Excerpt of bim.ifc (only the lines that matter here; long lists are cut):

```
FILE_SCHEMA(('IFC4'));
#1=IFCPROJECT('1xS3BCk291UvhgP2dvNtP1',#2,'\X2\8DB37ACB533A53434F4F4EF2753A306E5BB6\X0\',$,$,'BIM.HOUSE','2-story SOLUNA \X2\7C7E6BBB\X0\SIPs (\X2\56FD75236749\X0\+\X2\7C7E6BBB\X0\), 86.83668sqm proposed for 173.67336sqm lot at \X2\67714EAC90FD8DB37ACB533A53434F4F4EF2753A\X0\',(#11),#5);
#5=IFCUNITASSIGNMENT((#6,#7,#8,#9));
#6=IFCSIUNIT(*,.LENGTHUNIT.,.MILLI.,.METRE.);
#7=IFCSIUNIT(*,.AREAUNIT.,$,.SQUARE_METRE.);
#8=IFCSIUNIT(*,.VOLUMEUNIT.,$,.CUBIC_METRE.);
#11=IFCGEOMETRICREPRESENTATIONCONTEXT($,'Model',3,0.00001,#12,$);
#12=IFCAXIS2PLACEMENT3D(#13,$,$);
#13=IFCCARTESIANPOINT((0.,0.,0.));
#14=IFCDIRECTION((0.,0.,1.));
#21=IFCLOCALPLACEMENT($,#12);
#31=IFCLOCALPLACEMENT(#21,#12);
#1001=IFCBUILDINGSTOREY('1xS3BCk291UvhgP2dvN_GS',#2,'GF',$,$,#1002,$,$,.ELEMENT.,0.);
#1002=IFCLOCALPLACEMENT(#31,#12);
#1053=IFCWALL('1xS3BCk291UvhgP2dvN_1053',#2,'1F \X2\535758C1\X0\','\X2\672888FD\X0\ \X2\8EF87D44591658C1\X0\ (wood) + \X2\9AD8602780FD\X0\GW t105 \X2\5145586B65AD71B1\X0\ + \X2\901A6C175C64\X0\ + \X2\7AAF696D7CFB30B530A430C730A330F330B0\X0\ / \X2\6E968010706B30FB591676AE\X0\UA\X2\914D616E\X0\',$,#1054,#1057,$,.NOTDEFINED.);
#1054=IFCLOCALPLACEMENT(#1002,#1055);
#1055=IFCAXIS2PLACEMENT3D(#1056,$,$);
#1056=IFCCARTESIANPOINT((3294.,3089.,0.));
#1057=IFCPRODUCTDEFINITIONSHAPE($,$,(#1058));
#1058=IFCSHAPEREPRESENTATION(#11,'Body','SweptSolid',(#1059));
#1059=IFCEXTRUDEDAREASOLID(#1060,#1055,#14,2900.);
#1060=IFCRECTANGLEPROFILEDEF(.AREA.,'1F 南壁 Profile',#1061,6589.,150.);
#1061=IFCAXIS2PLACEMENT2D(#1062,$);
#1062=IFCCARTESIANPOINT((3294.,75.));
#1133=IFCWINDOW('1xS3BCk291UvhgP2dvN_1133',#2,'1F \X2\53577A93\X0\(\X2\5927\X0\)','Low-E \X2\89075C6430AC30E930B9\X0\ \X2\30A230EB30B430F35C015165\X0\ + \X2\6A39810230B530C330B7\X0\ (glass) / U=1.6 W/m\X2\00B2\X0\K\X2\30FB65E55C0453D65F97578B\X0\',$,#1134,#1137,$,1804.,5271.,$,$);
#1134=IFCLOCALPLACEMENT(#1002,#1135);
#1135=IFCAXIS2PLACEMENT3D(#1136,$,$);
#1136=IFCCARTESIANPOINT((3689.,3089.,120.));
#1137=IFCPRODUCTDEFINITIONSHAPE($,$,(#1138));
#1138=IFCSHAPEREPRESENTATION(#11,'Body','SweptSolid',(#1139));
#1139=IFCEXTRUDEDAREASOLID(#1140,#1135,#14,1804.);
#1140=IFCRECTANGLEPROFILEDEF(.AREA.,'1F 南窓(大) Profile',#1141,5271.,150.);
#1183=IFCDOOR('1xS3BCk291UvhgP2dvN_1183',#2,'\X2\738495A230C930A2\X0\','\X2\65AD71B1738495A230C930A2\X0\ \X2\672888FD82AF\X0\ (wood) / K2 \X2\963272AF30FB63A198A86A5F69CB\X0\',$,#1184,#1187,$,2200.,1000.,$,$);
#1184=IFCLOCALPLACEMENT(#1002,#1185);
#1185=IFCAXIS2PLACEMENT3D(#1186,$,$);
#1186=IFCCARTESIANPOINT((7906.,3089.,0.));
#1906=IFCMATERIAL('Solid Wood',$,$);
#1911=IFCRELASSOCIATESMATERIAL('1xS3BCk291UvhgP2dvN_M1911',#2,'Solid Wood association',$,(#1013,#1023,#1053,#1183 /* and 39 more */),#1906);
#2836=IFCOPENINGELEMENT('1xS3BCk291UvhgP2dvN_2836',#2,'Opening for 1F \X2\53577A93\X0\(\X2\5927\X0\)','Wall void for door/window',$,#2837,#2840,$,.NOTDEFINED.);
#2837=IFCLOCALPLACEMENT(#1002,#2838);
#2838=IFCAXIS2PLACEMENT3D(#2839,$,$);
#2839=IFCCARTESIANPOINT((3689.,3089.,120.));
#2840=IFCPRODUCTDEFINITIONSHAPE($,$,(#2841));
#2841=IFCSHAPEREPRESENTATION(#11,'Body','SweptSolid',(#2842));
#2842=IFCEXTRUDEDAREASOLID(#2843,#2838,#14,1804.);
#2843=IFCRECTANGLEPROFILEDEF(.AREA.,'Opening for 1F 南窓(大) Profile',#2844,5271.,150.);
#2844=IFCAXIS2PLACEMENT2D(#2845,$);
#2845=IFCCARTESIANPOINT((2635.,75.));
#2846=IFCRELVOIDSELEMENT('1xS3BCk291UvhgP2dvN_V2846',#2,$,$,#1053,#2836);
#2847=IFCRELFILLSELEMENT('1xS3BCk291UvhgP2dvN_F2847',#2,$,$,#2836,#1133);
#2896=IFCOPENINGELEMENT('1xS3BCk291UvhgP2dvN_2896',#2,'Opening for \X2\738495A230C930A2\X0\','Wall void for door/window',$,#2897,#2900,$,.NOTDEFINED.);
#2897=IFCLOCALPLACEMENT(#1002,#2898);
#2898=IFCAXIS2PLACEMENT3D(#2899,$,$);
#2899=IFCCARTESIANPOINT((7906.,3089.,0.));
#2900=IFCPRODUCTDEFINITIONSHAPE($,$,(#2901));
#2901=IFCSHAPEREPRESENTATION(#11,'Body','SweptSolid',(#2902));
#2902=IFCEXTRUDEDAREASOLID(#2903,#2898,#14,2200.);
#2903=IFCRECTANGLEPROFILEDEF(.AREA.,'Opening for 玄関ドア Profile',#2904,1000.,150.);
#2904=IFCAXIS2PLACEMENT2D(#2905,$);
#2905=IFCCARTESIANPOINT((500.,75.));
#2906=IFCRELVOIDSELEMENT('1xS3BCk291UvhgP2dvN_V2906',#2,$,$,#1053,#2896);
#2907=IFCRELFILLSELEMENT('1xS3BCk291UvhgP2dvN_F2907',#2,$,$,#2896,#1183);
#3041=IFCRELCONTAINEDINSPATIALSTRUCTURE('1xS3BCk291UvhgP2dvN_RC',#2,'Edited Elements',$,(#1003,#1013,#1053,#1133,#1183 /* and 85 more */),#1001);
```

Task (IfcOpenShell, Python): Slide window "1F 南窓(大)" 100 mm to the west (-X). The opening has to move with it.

```python
import ifcopenshell
import ifcopenshell.api.geometry
import ifcopenshell.util.placement

model = ifcopenshell.open("bim.ifc")

window = model.by_guid("1xS3BCk291UvhgP2dvN_1133")
opening = window.FillsVoids[0].RelatingOpeningElement
wall = opening.VoidsElements[0].RelatingBuildingElement

wall_matrix = ifcopenshell.util.placement.get_local_placement(wall.ObjectPlacement)
shift = wall_matrix[:3, 0] * -100.0
before = ifcopenshell.util.placement.get_local_placement(window.ObjectPlacement)[:3, 3].copy()

# The window is not placed relative to its opening, so move both.
for product in (opening, window):
    matrix = ifcopenshell.util.placement.get_local_placement(product.ObjectPlacement)
    matrix[:3, 3] += shift
    ifcopenshell.api.geometry.edit_object_placement(model, product=product, matrix=matrix, is_si=False)

after = ifcopenshell.util.placement.get_local_placement(window.ObjectPlacement)[:3, 3]
print("window moved by", (after - before).round(3) + 0.0)

model.write("bim_v2.ifc")
```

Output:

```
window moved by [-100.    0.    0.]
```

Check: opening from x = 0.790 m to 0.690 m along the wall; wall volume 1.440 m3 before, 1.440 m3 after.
